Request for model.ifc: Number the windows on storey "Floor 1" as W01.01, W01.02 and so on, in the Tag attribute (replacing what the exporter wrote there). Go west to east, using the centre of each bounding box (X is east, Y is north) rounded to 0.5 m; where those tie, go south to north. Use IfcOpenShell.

First a look at what the model holds.

```python
import ifcopenshell
import ifcopenshell.util.element
import ifcopenshell.util.placement

model = ifcopenshell.open("model.ifc")
print(model.schema)
storey = next(s for s in model.by_type("IfcBuildingStorey") if s.Name == "Floor 1")
windows = [e for e in ifcopenshell.util.element.get_decomposition(storey) if e.is_a("IfcWindow")]
for e in sorted(windows, key=lambda e: e.id()):
    origin = ifcopenshell.util.placement.get_local_placement(e.ObjectPlacement)[:3, 3]
    print(e.id(), e.Tag, e.Name, origin.round(2) + 0.0, sep=" | ")
```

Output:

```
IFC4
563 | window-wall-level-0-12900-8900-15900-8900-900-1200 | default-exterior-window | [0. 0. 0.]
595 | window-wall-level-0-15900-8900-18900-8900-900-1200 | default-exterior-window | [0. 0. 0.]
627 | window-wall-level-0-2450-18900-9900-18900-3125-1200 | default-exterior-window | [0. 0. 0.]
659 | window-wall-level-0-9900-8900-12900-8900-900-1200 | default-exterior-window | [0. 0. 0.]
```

```python
import ifcopenshell
import ifcopenshell.geom
import ifcopenshell.util.element
import ifcopenshell.util.shape

model = ifcopenshell.open("model.ifc")
settings = ifcopenshell.geom.settings()
settings.set("use-world-coords", True)


def centre(element):
    shape = ifcopenshell.geom.create_shape(settings, element)
    return ifcopenshell.util.shape.get_bbox_centroid(shape.geometry)


storey = next(s for s in model.by_type("IfcBuildingStorey") if s.Name == "Floor 1")
windows = [e for e in ifcopenshell.util.element.get_decomposition(storey) if e.is_a("IfcWindow")]

# Insertion points can sit at a corner or the storey origin, so sort by the geometry (in metres).
centres = {e: centre(e) for e in windows}
windows.sort(key=lambda e: (round(centres[e][0] / 0.5), centres[e][1]))

for i, e in enumerate(windows, start=1):
    number = f"W01.{i:02d}"
    e.Tag = number
    print(e.id(), number)

model.write("model_rev.ifc")
```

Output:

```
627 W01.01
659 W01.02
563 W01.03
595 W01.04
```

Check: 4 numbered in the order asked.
